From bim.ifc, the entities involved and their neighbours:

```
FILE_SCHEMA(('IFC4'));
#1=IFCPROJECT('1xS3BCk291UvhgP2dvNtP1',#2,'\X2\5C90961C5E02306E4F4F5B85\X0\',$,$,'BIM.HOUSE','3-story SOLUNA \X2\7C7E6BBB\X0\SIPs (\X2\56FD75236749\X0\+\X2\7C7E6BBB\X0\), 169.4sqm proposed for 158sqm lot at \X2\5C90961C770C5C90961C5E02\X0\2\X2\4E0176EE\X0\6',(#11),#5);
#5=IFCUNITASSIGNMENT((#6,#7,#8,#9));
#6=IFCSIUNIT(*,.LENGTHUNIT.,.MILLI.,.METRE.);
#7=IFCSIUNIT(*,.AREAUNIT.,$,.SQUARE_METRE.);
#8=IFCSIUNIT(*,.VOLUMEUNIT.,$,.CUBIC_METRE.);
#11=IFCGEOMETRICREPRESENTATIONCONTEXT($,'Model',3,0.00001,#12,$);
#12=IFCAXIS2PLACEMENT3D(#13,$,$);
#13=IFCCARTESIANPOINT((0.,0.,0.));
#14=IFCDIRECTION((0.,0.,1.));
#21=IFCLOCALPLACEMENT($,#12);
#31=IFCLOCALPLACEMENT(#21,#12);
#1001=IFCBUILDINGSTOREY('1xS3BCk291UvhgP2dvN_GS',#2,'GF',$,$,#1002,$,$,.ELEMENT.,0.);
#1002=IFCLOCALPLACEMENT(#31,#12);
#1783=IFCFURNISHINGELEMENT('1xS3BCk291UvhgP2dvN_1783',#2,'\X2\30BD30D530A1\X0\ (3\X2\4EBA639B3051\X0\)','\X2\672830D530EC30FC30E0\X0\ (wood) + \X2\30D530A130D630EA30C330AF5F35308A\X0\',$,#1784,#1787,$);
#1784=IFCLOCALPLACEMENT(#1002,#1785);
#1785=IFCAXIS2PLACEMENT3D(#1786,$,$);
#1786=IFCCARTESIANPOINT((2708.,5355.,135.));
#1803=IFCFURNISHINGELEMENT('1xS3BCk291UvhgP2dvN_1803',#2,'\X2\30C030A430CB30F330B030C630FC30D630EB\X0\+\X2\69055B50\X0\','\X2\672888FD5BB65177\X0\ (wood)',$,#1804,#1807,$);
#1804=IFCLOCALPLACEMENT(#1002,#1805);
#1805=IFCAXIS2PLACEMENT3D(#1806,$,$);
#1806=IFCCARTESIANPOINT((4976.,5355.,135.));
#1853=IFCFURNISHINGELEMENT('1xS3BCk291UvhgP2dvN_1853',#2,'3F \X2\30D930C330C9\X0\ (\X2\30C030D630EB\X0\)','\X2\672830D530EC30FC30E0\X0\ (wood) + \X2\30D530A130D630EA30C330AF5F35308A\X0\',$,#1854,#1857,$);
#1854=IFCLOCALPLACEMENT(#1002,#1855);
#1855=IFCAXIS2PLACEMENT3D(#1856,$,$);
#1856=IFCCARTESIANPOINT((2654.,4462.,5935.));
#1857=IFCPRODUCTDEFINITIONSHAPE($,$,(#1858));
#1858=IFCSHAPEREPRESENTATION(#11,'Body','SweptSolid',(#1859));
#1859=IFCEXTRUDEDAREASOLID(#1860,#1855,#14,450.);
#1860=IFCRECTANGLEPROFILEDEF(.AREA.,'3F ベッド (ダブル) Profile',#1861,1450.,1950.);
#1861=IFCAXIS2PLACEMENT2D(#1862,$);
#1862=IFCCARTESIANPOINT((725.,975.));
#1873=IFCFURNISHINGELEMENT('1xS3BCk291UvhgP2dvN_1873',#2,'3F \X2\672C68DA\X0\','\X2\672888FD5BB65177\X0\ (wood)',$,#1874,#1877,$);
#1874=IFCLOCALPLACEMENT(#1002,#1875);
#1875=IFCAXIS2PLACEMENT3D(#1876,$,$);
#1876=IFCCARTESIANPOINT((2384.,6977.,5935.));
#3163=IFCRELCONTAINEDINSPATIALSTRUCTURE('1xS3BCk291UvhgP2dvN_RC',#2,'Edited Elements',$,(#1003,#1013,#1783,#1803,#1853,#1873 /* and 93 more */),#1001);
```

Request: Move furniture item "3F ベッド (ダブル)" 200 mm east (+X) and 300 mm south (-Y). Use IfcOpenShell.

```python
import ifcopenshell
import ifcopenshell.api.geometry
import ifcopenshell.util.placement

model = ifcopenshell.open("bim.ifc")

item = model.by_guid("1xS3BCk291UvhgP2dvN_1853")
matrix = ifcopenshell.util.placement.get_local_placement(item.ObjectPlacement)
matrix[0, 3] += 200.0
matrix[1, 3] -= 300.0
ifcopenshell.api.geometry.edit_object_placement(model, product=item, matrix=matrix, is_si=False)

print(ifcopenshell.util.placement.get_local_placement(item.ObjectPlacement).round(3) + 0.0)

model.write("bim-out.ifc")
```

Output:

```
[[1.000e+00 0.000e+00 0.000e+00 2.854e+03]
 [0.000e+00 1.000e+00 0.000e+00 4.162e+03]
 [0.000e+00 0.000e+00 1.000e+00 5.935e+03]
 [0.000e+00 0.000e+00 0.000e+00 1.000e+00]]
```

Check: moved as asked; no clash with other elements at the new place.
